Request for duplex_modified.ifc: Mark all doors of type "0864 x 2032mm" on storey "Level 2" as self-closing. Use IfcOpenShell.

First a look at what the model holds.

```python
import ifcopenshell
import ifcopenshell.util.element

model = ifcopenshell.open("duplex_modified.ifc")
print(model.schema)
storey = next(s for s in model.by_type("IfcBuildingStorey") if s.Name == "Level 2")
doors = [e for e in ifcopenshell.util.element.get_decomposition(storey) if e.is_a("IfcDoor")]
seen = {}
for e in doors:
    element_type = ifcopenshell.util.element.get_type(e)
    key = (element_type.Name if element_type != e and element_type else None, ifcopenshell.util.element.get_pset(e, "Pset_DoorCommon", "SelfClosing"))
    seen[key] = seen.get(key, 0) + 1
for (name, value), count in sorted(seen.items(), key=str):
    print(count, "x", name, "|", value)
```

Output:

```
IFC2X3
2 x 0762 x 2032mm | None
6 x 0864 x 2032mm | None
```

```python
import ifcopenshell
import ifcopenshell.api.pset
import ifcopenshell.util.element

model = ifcopenshell.open("duplex_modified.ifc")

storey = next(s for s in model.by_type("IfcBuildingStorey") if s.Name == "Level 2")
doors = [e for e in ifcopenshell.util.element.get_decomposition(storey) if e.is_a("IfcDoor")]

count = 0
for e in doors:
    element_type = ifcopenshell.util.element.get_type(e)
    if element_type in (None, e) or element_type.Name != "0864 x 2032mm":
        continue
    # add_pset returns the element's existing set when there is one.
    pset = ifcopenshell.api.pset.add_pset(model, product=e, name="Pset_DoorCommon")
    ifcopenshell.api.pset.edit_pset(model, pset=pset, properties={"SelfClosing": True})
    count += 1

print(count, "doors updated")

model.write("duplex_modified_v2.ifc")
```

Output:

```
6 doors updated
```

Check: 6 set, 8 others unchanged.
